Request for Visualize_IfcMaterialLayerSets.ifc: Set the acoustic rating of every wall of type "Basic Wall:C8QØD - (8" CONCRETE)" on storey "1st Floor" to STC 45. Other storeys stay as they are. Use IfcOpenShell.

First a look at what the model holds.

```python
import ifcopenshell
import ifcopenshell.util.element

model = ifcopenshell.open("Visualize_IfcMaterialLayerSets.ifc")
print(model.schema)
storey = next(s for s in model.by_type("IfcBuildingStorey") if s.Name == "1st Floor")
walls = [e for e in ifcopenshell.util.element.get_decomposition(storey) if e.is_a("IfcWall")]
seen = {}
for e in walls:
    element_type = ifcopenshell.util.element.get_type(e)
    key = (element_type.Name if element_type != e and element_type else None, ifcopenshell.util.element.get_pset(e, "Pset_WallCommon", "AcousticRating"))
    seen[key] = seen.get(key, 0) + 1
for (name, value), count in sorted(seen.items(), key=str):
    print(count, "x", name, "|", value)
```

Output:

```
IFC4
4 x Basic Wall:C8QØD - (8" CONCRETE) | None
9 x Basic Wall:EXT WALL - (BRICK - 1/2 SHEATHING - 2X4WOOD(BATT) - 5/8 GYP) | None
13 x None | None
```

```python
import ifcopenshell
import ifcopenshell.api.pset
import ifcopenshell.util.element

model = ifcopenshell.open("Visualize_IfcMaterialLayerSets.ifc")

storey = next(s for s in model.by_type("IfcBuildingStorey") if s.Name == "1st Floor")
walls = [e for e in ifcopenshell.util.element.get_decomposition(storey) if e.is_a("IfcWall")]

count = 0
for e in walls:
    element_type = ifcopenshell.util.element.get_type(e)
    if element_type in (None, e) or element_type.Name != 'Basic Wall:C8QØD - (8" CONCRETE)':
        continue
    # add_pset returns the element's existing set when there is one.
    pset = ifcopenshell.api.pset.add_pset(model, product=e, name="Pset_WallCommon")
    ifcopenshell.api.pset.edit_pset(model, pset=pset, properties={"AcousticRating": "STC 45"})
    count += 1

print(count, "walls updated")

model.write("Visualize_IfcMaterialLayerSets_v2.ifc")
```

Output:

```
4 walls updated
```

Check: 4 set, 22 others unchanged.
